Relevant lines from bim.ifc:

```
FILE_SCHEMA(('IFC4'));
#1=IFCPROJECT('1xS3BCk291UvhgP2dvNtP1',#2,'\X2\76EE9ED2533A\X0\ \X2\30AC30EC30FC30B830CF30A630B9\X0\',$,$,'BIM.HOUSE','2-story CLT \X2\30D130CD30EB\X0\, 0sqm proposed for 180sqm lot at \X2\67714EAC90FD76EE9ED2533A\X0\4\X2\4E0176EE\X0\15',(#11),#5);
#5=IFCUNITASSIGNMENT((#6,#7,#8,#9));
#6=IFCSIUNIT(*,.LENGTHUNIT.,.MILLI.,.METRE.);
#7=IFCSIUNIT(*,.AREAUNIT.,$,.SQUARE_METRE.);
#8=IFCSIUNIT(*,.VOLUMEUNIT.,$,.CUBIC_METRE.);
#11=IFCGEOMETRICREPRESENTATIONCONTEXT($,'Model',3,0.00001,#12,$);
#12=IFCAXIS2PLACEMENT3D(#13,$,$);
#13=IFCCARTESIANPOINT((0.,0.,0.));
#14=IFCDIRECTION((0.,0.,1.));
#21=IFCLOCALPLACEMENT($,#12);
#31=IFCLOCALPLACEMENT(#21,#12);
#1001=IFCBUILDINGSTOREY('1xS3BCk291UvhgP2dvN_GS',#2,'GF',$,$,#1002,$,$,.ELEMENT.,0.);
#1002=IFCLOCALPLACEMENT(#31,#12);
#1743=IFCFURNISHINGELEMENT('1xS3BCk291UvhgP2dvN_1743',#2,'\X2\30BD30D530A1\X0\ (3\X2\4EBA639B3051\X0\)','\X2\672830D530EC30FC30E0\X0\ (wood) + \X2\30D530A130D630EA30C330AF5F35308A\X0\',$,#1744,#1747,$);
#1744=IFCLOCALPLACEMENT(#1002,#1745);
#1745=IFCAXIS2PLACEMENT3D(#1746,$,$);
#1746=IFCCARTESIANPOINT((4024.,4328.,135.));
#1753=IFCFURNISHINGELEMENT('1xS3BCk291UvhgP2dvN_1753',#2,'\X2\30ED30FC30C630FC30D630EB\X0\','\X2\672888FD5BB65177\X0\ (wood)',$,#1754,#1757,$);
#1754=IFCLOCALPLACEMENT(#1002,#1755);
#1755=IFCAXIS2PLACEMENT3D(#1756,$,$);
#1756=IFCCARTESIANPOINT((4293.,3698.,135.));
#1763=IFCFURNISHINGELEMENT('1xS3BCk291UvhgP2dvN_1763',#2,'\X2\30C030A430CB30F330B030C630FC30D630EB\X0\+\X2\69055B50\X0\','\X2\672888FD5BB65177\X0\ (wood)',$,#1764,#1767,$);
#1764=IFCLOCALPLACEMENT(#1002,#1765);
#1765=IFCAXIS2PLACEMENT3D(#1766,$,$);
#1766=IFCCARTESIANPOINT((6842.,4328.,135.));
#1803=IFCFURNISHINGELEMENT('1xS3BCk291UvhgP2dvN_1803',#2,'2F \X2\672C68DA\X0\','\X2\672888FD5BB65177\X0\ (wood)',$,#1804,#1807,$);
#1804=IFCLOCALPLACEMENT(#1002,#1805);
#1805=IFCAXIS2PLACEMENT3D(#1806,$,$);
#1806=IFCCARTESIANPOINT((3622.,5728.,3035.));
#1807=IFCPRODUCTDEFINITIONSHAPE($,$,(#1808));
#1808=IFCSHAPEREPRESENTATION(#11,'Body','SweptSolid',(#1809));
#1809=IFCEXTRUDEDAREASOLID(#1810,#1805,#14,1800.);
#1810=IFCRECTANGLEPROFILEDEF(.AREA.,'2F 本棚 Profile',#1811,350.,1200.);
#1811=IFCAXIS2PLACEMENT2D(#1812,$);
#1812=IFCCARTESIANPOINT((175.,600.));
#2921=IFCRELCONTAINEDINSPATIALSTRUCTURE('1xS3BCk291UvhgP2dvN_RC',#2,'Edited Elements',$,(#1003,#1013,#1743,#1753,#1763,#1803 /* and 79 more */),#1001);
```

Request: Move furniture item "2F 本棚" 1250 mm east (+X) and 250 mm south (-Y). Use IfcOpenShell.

```python
import ifcopenshell
import ifcopenshell.api.geometry
import ifcopenshell.util.placement
import ifcopenshell.util.unit

model = ifcopenshell.open("bim.ifc")
unit_scale = ifcopenshell.util.unit.calculate_unit_scale(model)

item = model.by_id(1803)
matrix = ifcopenshell.util.placement.get_local_placement(item.ObjectPlacement)
matrix[0, 3] += 1.25 / unit_scale
matrix[1, 3] -= 0.25 / unit_scale
ifcopenshell.api.geometry.edit_object_placement(model, product=item, matrix=matrix, is_si=False)

print(ifcopenshell.util.placement.get_local_placement(item.ObjectPlacement).round(3) + 0.0)

model.write("bim_updated.ifc")
```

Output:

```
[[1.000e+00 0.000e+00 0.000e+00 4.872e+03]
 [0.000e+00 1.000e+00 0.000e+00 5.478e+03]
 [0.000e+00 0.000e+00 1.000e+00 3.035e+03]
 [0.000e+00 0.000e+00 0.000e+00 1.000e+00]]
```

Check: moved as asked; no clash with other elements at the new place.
